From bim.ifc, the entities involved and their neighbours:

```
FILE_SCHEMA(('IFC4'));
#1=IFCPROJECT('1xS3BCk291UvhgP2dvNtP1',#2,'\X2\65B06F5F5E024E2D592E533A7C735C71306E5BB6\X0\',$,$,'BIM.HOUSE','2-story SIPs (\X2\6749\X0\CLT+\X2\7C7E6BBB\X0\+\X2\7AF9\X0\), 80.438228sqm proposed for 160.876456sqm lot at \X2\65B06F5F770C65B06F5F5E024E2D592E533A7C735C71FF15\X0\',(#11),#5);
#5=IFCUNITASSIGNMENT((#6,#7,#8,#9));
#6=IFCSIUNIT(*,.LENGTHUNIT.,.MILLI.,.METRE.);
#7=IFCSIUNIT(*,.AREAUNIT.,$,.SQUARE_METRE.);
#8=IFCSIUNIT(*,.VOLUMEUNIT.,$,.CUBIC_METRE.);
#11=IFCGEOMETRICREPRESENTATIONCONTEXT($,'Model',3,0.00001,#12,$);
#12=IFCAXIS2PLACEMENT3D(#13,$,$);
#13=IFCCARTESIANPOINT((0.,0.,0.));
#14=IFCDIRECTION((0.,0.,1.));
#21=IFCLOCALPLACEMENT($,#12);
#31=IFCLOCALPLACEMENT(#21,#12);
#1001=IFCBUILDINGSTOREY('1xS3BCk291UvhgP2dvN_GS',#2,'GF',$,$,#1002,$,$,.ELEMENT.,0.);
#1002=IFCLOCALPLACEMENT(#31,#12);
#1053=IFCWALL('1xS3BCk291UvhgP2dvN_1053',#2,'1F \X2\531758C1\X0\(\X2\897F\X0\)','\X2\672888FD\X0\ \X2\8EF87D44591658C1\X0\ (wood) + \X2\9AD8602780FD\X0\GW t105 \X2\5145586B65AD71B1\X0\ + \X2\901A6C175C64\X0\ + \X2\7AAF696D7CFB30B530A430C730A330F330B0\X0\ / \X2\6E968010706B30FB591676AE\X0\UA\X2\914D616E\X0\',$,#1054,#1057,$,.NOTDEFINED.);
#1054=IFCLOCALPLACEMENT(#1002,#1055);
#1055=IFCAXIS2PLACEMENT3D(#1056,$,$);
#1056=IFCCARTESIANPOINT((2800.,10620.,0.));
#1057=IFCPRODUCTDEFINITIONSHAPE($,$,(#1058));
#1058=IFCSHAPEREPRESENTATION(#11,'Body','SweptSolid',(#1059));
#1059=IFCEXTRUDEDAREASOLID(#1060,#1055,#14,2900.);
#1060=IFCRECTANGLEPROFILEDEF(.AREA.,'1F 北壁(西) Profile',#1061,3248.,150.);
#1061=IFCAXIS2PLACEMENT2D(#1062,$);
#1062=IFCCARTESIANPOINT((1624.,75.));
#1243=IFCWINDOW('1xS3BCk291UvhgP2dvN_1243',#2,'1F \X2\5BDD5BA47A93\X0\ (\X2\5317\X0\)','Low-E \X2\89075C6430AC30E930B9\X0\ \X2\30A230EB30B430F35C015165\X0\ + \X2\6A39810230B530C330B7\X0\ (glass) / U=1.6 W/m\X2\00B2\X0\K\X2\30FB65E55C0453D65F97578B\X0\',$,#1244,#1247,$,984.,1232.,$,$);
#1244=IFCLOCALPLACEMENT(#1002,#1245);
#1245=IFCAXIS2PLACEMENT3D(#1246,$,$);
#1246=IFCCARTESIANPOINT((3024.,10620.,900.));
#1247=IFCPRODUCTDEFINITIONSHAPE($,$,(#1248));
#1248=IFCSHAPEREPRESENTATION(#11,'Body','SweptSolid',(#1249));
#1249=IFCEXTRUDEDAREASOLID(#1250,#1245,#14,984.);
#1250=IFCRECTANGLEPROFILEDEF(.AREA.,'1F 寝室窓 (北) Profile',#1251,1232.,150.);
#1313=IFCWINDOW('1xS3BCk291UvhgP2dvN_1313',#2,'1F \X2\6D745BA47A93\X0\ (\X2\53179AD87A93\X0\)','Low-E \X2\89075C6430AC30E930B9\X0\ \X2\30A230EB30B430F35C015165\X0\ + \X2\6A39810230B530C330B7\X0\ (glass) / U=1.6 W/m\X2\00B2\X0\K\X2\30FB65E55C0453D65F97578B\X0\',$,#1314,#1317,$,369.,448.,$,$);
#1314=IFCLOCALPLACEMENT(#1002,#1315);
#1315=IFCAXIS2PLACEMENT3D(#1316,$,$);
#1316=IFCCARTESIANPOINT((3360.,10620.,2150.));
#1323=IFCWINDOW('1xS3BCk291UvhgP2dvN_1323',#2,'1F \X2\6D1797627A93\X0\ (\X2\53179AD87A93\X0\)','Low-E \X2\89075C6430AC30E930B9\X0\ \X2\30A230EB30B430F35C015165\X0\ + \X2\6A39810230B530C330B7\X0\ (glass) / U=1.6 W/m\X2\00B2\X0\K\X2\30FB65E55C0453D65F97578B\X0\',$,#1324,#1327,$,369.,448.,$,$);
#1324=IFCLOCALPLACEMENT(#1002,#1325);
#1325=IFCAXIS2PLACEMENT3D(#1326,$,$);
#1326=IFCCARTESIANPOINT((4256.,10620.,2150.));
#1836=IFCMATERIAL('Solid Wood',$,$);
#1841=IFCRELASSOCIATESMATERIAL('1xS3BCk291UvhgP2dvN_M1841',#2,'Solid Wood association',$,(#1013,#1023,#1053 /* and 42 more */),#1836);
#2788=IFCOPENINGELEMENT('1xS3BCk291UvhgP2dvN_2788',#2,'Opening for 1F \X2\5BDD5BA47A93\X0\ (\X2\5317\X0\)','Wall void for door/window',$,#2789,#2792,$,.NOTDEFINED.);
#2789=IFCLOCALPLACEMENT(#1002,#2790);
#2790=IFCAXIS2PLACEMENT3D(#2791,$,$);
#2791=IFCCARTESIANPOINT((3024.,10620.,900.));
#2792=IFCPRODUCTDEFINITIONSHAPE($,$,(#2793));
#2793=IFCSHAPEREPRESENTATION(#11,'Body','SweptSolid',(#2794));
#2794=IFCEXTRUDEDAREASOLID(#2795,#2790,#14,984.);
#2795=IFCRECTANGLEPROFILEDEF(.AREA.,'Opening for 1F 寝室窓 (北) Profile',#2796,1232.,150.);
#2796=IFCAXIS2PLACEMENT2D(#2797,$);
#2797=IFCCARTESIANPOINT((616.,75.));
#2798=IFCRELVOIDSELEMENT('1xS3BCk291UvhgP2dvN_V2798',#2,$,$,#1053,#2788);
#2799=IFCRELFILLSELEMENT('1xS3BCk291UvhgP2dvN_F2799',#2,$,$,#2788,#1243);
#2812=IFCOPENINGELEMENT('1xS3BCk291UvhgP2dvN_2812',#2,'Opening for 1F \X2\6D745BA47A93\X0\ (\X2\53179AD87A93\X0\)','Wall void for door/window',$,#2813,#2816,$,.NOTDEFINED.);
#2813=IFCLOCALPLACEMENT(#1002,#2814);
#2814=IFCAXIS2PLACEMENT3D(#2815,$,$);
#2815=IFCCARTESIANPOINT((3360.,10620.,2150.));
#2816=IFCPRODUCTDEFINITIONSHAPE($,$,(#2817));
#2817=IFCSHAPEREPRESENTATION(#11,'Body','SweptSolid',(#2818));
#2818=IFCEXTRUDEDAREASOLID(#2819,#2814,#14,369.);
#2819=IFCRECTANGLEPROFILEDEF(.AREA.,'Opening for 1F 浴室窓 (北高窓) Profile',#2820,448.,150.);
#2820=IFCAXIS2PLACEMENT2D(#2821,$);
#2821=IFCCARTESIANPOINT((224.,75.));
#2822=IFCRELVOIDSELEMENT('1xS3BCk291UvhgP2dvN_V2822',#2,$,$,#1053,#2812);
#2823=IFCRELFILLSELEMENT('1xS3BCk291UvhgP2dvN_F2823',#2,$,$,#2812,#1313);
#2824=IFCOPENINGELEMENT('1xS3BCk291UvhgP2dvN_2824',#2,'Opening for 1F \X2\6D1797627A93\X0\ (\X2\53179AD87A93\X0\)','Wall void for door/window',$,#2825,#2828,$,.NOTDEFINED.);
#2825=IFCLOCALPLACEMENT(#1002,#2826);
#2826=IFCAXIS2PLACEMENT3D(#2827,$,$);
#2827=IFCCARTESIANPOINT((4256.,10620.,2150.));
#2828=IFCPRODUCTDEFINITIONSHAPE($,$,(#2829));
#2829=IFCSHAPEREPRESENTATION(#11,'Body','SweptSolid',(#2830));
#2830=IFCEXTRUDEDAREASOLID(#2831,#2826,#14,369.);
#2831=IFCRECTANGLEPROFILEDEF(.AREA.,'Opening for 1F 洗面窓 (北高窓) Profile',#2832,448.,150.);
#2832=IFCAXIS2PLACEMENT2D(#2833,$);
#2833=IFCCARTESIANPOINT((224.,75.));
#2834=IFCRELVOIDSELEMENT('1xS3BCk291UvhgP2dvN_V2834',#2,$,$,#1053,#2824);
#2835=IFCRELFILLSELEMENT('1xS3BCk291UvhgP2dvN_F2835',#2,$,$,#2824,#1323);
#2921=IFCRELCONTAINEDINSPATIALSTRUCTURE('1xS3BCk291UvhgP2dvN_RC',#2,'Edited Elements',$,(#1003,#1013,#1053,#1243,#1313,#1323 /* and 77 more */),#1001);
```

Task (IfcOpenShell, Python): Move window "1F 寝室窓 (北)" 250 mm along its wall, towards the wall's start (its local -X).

```python
import ifcopenshell
import ifcopenshell.api.geometry
import ifcopenshell.util.placement
import ifcopenshell.util.unit

model = ifcopenshell.open("bim.ifc")
unit_scale = ifcopenshell.util.unit.calculate_unit_scale(model)

window = model.by_guid("1xS3BCk291UvhgP2dvN_1243")
opening = window.FillsVoids[0].RelatingOpeningElement
wall = opening.VoidsElements[0].RelatingBuildingElement

wall_matrix = ifcopenshell.util.placement.get_local_placement(wall.ObjectPlacement)
shift = wall_matrix[:3, 0] * -0.25 / unit_scale
before = ifcopenshell.util.placement.get_local_placement(window.ObjectPlacement)[:3, 3].copy()

# The window is not placed relative to its opening, so move both.
for product in (opening, window):
    matrix = ifcopenshell.util.placement.get_local_placement(product.ObjectPlacement)
    matrix[:3, 3] += shift
    ifcopenshell.api.geometry.edit_object_placement(model, product=product, matrix=matrix, is_si=False)

after = ifcopenshell.util.placement.get_local_placement(window.ObjectPlacement)[:3, 3]
print("window moved by", (after - before).round(3) + 0.0)

model.write("bim_rev.ifc")
```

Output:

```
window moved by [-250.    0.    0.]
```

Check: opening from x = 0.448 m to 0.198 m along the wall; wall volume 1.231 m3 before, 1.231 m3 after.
